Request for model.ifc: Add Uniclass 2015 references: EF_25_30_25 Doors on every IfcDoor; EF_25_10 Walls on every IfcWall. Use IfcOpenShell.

First a look at what the model holds.

```python
import ifcopenshell

model = ifcopenshell.open("model.ifc")
print(model.schema)
print("classifications:", [c.Name for c in model.by_type("IfcClassification")])
for ifc_class in ("IfcDoor", "IfcRoof", "IfcStair", "IfcWall", "IfcWindow"):
    print(ifc_class, len(model.by_type(ifc_class)))
```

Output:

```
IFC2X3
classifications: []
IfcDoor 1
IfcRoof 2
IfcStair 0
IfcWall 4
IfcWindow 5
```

```python
import ifcopenshell
import ifcopenshell.api.classification

model = ifcopenshell.open("model.ifc")

# IFC2X3 requires Source and Edition and has no link from the project to the system.
system = model.create_entity("IfcClassification", Source="NBS", Edition="2015", Name="Uniclass 2015")

codes = {
    "IfcDoor": ("EF_25_30_25", "Doors"),
    "IfcWall": ("EF_25_10", "Walls"),
}
for ifc_class, (code, name) in codes.items():
    products = model.by_type(ifc_class)
    ifcopenshell.api.classification.add_reference(
        model, products=products, classification=system, identification=code, name=name
    )
    print(code, len(products))

model.write("model_updated.ifc")
```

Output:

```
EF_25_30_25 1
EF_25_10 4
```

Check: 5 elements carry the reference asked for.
